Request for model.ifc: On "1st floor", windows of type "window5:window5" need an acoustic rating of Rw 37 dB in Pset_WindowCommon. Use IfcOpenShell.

First a look at what the model holds.

```python
import ifcopenshell
import ifcopenshell.util.element

model = ifcopenshell.open("model.ifc")
print(model.schema)
storey = next(s for s in model.by_type("IfcBuildingStorey") if s.Name == "1st floor")
windows = [e for e in ifcopenshell.util.element.get_decomposition(storey) if e.is_a("IfcWindow")]
seen = {}
for e in windows:
    element_type = ifcopenshell.util.element.get_type(e)
    key = (element_type.Name if element_type != e and element_type else None, ifcopenshell.util.element.get_pset(e, "Pset_WindowCommon", "AcousticRating"))
    seen[key] = seen.get(key, 0) + 1
for (name, value), count in sorted(seen.items(), key=str):
    print(count, "x", name, "|", value)
```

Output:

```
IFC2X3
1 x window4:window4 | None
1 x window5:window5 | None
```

```python
import ifcopenshell
import ifcopenshell.api.pset
import ifcopenshell.util.element

model = ifcopenshell.open("model.ifc")

storey = next(s for s in model.by_type("IfcBuildingStorey") if s.Name == "1st floor")
windows = [e for e in ifcopenshell.util.element.get_decomposition(storey) if e.is_a("IfcWindow")]

count = 0
for e in windows:
    element_type = ifcopenshell.util.element.get_type(e)
    if element_type in (None, e) or element_type.Name != "window5:window5":
        continue
    # add_pset returns the element's existing set when there is one.
    pset = ifcopenshell.api.pset.add_pset(model, product=e, name="Pset_WindowCommon")
    ifcopenshell.api.pset.edit_pset(model, pset=pset, properties={"AcousticRating": "Rw 37 dB"})
    count += 1

print(count, "windows updated")

model.write("model_updated.ifc")
```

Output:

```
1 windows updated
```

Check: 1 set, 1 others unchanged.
